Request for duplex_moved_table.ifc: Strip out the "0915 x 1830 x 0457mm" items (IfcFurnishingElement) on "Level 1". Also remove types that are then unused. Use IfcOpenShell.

First a look at what the model holds.

```python
import ifcopenshell
import ifcopenshell.util.element

model = ifcopenshell.open("duplex_moved_table.ifc")
print(model.schema)
storey = next(s for s in model.by_type("IfcBuildingStorey") if s.Name == "Level 1")
furniture = [e for e in ifcopenshell.util.element.get_decomposition(storey) if e.is_a("IfcFurnishingElement")]
seen = {}
for e in furniture:
    element_type = ifcopenshell.util.element.get_type(e)
    name = element_type.Name if element_type not in (None, e) else None
    seen[name] = seen.get(name, 0) + 1
for name, count in sorted(seen.items(), key=str):
    print(count, "x", name)
```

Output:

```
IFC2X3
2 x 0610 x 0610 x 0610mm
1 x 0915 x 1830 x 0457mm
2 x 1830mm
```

```python
import ifcopenshell
import ifcopenshell.api.root
import ifcopenshell.util.element

model = ifcopenshell.open("duplex_moved_table.ifc")

storey = next(s for s in model.by_type("IfcBuildingStorey") if s.Name == "Level 1")
furniture = [e for e in ifcopenshell.util.element.get_decomposition(storey) if e.is_a("IfcFurnishingElement")]
targets = [e for e in furniture if (t := ifcopenshell.util.element.get_type(e)) not in (None, e) and t.Name == "0915 x 1830 x 0457mm"]
types = {ifcopenshell.util.element.get_type(e) for e in targets} - {None, *targets}

for e in targets:
    ifcopenshell.api.root.remove_product(model, product=e)
print(len(targets), "removed")

unused = [t for t in types if not ifcopenshell.util.element.get_types(t)]
for t in unused:
    ifcopenshell.api.root.remove_product(model, product=t)
print(len(unused), "unused types removed")

model.write("duplex_moved_table_v2.ifc")
```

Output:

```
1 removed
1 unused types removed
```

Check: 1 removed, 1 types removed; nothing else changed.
